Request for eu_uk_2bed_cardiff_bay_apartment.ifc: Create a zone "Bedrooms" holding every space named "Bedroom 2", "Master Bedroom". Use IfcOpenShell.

First a look at what the model holds.

```python
import ifcopenshell

model = ifcopenshell.open("eu_uk_2bed_cardiff_bay_apartment.ifc")
print(model.schema)
seen = {}
for space in model.by_type("IfcSpace"):
    seen[space.LongName] = seen.get(space.LongName, 0) + 1
for name, count in sorted(seen.items(), key=str):
    print(count, "x", name)
print("zones:", [z.Name for z in model.by_type("IfcZone")][:20])
```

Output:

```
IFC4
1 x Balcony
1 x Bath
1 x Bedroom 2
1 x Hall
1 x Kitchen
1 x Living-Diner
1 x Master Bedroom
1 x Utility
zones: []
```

```python
import ifcopenshell
import ifcopenshell.api.group
import ifcopenshell.api.root

model = ifcopenshell.open("eu_uk_2bed_cardiff_bay_apartment.ifc")

names = {"Bedroom 2", "Master Bedroom"}
spaces = [s for s in model.by_type("IfcSpace") if s.LongName in names]

zone = ifcopenshell.api.root.create_entity(model, ifc_class="IfcZone", name="Bedrooms")
ifcopenshell.api.group.assign_group(model, products=spaces, group=zone)
print(len(spaces), "spaces in", zone.Name)

model.write("eu_uk_2bed_cardiff_bay_apartment_v2.ifc")
```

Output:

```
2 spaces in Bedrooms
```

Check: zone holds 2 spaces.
